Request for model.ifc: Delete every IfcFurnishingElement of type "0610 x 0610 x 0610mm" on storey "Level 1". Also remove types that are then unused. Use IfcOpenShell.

First a look at what the model holds.

```python
import ifcopenshell
import ifcopenshell.util.element

model = ifcopenshell.open("model.ifc")
print(model.schema)
storey = next(s for s in model.by_type("IfcBuildingStorey") if s.Name == "Level 1")
furniture = [e for e in ifcopenshell.util.element.get_decomposition(storey) if e.is_a("IfcFurnishingElement")]
seen = {}
for e in furniture:
    element_type = ifcopenshell.util.element.get_type(e)
    name = element_type.Name if element_type not in (None, e) else None
    seen[name] = seen.get(name, 0) + 1
for name, count in sorted(seen.items(), key=str):
    print(count, "x", name)
```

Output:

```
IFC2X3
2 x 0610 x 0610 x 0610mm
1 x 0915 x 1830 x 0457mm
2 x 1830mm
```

```python
import ifcopenshell
import ifcopenshell.api.root
import ifcopenshell.util.element

model = ifcopenshell.open("model.ifc")

storey = next(s for s in model.by_type("IfcBuildingStorey") if s.Name == "Level 1")
furniture = [e for e in ifcopenshell.util.element.get_decomposition(storey) if e.is_a("IfcFurnishingElement")]
targets = [e for e in furniture if (t := ifcopenshell.util.element.get_type(e)) not in (None, e) and t.Name == "0610 x 0610 x 0610mm"]
types = {ifcopenshell.util.element.get_type(e) for e in targets} - {None, *targets}

for e in targets:
    ifcopenshell.api.root.remove_product(model, product=e)
print(len(targets), "removed")

unused = [t for t in types if not ifcopenshell.util.element.get_types(t)]
for t in unused:
    ifcopenshell.api.root.remove_product(model, product=t)
print(len(unused), "unused types removed")

model.write("model_v2.ifc")
```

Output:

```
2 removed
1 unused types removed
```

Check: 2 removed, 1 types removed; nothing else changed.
